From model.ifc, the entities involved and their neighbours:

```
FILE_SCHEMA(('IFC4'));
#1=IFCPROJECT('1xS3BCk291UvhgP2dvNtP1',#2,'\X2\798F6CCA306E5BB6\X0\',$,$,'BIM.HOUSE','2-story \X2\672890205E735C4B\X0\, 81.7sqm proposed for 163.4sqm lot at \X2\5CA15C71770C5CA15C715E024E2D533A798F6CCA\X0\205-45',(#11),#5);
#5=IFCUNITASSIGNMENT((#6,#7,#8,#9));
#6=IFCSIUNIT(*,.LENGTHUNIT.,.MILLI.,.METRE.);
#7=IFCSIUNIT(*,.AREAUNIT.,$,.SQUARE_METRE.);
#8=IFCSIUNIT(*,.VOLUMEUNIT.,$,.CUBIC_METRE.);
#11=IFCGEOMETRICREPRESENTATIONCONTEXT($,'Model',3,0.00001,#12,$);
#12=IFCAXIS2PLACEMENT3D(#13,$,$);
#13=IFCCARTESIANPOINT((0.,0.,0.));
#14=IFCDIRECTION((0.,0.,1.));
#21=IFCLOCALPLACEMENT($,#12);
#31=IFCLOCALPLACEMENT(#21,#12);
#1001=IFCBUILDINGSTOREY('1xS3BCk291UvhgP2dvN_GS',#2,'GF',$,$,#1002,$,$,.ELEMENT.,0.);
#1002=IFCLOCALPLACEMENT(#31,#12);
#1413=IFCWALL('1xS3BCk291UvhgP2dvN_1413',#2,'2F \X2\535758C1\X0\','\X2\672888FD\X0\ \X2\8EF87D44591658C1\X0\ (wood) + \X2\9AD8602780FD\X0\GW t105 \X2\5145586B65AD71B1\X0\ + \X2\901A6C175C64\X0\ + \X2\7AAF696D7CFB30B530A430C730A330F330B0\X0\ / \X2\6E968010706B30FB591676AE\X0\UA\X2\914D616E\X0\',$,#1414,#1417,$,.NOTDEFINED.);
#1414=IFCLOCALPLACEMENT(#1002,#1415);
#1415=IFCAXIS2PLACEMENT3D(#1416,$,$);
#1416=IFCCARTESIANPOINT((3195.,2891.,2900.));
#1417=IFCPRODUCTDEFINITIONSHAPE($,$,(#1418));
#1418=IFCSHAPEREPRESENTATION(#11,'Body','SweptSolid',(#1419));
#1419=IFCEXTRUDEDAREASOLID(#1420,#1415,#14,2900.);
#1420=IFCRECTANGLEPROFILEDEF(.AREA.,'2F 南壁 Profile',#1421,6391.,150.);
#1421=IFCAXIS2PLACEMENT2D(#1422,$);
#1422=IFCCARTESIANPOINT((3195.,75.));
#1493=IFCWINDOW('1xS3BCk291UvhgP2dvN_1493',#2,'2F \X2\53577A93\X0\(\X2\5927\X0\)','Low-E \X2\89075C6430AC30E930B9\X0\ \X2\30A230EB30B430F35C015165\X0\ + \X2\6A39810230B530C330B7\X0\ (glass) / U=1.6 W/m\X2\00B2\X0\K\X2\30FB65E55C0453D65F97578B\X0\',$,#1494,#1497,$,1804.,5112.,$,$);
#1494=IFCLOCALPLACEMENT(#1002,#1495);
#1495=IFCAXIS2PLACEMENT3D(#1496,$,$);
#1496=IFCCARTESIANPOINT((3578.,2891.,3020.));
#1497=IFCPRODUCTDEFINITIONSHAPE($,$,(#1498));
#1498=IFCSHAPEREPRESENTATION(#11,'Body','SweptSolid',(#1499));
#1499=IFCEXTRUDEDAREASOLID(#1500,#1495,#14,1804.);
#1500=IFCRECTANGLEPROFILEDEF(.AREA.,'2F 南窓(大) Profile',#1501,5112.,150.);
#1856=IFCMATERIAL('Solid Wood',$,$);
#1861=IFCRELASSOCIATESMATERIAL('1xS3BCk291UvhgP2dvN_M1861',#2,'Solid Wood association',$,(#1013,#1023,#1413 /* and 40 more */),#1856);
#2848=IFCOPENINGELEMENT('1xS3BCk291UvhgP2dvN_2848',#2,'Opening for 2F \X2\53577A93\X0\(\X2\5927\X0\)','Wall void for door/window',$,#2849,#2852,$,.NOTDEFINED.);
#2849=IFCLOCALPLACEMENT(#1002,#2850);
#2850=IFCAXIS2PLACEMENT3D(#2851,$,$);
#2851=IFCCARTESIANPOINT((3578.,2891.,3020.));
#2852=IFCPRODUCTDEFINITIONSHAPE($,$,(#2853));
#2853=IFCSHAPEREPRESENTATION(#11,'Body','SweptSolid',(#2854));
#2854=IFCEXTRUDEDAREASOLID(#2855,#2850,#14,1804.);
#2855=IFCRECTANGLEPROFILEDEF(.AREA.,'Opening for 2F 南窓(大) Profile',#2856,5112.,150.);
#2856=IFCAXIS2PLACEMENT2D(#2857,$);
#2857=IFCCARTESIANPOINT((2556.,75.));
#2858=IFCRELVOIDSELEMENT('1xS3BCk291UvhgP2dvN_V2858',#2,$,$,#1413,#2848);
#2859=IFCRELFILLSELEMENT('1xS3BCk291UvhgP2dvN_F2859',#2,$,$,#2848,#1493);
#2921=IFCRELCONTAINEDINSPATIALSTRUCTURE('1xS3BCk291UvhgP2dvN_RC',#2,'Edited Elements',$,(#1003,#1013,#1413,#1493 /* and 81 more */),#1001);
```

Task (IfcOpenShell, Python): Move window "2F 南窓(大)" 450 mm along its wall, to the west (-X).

```python
import ifcopenshell
import ifcopenshell.api.geometry
import ifcopenshell.util.placement
import ifcopenshell.util.unit

model = ifcopenshell.open("model.ifc")
unit_scale = ifcopenshell.util.unit.calculate_unit_scale(model)

window = model.by_guid("1xS3BCk291UvhgP2dvN_1493")
opening = window.FillsVoids[0].RelatingOpeningElement
wall = opening.VoidsElements[0].RelatingBuildingElement

wall_matrix = ifcopenshell.util.placement.get_local_placement(wall.ObjectPlacement)
shift = wall_matrix[:3, 0] * -0.45 / unit_scale
before = ifcopenshell.util.placement.get_local_placement(window.ObjectPlacement)[:3, 3].copy()

# The window is not placed relative to its opening, so move both.
for product in (opening, window):
    matrix = ifcopenshell.util.placement.get_local_placement(product.ObjectPlacement)
    matrix[:3, 3] += shift
    ifcopenshell.api.geometry.edit_object_placement(model, product=product, matrix=matrix, is_si=False)

after = ifcopenshell.util.placement.get_local_placement(window.ObjectPlacement)[:3, 3]
print("window moved by", (after - before).round(3) + 0.0)

model.write("model_edited.ifc")
```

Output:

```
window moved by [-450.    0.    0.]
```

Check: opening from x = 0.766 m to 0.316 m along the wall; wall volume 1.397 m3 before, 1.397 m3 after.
